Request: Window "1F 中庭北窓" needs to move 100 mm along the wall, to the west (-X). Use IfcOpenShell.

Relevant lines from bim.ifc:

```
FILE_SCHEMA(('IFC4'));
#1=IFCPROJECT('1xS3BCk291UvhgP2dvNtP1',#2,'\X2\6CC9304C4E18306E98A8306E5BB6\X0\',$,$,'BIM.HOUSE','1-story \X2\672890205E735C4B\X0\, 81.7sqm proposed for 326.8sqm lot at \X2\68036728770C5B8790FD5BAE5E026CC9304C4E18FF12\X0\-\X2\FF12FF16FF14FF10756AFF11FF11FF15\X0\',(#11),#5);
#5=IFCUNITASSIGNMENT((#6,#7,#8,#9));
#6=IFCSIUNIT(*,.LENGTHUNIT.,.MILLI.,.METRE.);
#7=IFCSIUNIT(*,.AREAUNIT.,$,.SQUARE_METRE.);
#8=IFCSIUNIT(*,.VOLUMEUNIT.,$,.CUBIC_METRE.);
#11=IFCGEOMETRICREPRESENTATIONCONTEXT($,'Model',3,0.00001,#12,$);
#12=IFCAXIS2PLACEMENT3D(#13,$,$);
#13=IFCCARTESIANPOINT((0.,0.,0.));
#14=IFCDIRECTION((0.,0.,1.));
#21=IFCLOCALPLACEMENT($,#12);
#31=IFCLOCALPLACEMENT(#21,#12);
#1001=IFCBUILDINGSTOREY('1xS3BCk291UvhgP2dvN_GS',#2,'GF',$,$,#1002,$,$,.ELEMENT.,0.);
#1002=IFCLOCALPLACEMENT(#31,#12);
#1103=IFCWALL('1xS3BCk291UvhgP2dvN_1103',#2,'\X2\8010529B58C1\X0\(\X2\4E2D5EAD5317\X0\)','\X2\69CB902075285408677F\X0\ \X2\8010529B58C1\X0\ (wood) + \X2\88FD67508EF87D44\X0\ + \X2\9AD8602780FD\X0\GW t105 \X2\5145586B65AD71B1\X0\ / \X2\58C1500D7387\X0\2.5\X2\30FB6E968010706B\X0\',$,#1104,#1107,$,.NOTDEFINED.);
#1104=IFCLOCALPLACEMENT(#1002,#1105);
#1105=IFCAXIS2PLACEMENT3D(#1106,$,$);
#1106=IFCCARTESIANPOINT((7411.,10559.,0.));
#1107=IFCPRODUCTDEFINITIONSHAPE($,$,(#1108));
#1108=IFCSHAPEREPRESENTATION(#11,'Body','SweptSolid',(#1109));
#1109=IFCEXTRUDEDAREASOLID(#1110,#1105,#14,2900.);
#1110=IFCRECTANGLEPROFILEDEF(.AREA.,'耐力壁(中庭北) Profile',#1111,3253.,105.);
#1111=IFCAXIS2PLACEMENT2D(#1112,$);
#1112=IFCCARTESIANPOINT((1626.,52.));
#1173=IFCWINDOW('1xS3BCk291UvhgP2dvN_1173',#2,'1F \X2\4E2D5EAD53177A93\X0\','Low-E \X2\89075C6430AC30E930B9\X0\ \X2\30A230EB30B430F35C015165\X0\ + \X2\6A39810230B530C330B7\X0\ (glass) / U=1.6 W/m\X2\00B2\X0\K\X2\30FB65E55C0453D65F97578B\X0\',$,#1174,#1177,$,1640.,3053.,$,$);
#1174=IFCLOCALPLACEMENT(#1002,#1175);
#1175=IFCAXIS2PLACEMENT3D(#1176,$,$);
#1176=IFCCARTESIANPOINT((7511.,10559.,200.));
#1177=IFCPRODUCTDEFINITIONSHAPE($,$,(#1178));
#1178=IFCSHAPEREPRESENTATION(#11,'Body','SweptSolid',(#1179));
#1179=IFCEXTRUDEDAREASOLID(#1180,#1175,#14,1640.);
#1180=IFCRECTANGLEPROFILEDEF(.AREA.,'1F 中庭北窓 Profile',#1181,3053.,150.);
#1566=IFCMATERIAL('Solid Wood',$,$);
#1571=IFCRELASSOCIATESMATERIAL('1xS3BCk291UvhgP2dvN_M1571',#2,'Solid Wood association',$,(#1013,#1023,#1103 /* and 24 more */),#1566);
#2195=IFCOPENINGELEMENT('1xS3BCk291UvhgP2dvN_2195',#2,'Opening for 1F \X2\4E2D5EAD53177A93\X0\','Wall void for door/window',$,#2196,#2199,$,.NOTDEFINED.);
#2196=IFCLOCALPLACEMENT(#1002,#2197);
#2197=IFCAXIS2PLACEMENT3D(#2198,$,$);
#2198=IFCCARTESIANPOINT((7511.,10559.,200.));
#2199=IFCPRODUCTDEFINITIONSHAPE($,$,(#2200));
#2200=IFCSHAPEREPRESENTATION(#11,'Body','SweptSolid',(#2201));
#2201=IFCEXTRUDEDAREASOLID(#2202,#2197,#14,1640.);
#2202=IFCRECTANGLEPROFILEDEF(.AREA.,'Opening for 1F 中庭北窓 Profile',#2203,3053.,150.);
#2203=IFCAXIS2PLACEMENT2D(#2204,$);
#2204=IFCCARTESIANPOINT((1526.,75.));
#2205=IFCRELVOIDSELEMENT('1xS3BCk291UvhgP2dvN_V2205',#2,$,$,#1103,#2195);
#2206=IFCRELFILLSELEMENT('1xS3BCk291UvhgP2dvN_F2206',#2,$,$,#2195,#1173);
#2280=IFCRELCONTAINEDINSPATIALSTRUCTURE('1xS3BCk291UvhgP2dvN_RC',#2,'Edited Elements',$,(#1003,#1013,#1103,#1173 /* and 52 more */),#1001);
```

```python
import ifcopenshell
import ifcopenshell.api.geometry
import ifcopenshell.util.placement

model = ifcopenshell.open("bim.ifc")

window = model.by_guid("1xS3BCk291UvhgP2dvN_1173")
opening = window.FillsVoids[0].RelatingOpeningElement
wall = opening.VoidsElements[0].RelatingBuildingElement

wall_matrix = ifcopenshell.util.placement.get_local_placement(wall.ObjectPlacement)
shift = wall_matrix[:3, 0] * -100.0
before = ifcopenshell.util.placement.get_local_placement(window.ObjectPlacement)[:3, 3].copy()

# The window is not placed relative to its opening, so move both.
for product in (opening, window):
    matrix = ifcopenshell.util.placement.get_local_placement(product.ObjectPlacement)
    matrix[:3, 3] += shift
    ifcopenshell.api.geometry.edit_object_placement(model, product=product, matrix=matrix, is_si=False)

after = ifcopenshell.util.placement.get_local_placement(window.ObjectPlacement)[:3, 3]
print("window moved by", (after - before).round(3) + 0.0)

model.write("bim_updated.ifc")
```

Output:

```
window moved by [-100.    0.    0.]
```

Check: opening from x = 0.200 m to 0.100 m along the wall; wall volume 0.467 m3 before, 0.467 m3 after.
